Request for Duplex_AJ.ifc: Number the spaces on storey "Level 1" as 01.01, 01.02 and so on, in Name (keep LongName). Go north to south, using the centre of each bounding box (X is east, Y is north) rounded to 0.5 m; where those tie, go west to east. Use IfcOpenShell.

First a look at what the model holds.

```python
import ifcopenshell
import ifcopenshell.util.element
import ifcopenshell.util.placement

model = ifcopenshell.open("Duplex_AJ.ifc")
print(model.schema)
storey = next(s for s in model.by_type("IfcBuildingStorey") if s.Name == "Level 1")
spaces = [e for e in ifcopenshell.util.element.get_decomposition(storey) if e.is_a("IfcSpace")]
for e in sorted(spaces, key=lambda e: e.id()):
    origin = ifcopenshell.util.placement.get_local_placement(e.ObjectPlacement)[:3, 3]
    print(e.id(), e.Name, e.LongName, origin.round(2) + 0.0, sep=" | ")
```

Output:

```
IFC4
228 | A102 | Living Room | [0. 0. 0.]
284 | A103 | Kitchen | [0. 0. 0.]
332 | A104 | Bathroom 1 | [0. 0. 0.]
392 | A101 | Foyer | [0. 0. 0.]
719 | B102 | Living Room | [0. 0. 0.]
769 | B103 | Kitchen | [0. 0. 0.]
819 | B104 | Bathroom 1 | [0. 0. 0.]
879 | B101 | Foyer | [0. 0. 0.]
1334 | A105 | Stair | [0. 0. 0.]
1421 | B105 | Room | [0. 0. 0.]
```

```python
import ifcopenshell
import ifcopenshell.geom
import ifcopenshell.util.element
import ifcopenshell.util.shape

model = ifcopenshell.open("Duplex_AJ.ifc")
settings = ifcopenshell.geom.settings()
settings.set("use-world-coords", True)


def centre(element):
    shape = ifcopenshell.geom.create_shape(settings, element)
    return ifcopenshell.util.shape.get_bbox_centroid(shape.geometry)


storey = next(s for s in model.by_type("IfcBuildingStorey") if s.Name == "Level 1")
spaces = [e for e in ifcopenshell.util.element.get_decomposition(storey) if e.is_a("IfcSpace")]

# Insertion points can sit at a corner or the storey origin, so sort by the geometry (in metres).
centres = {e: centre(e) for e in spaces}
spaces.sort(key=lambda e: (-round(centres[e][1] / 0.5), centres[e][0]))

for i, e in enumerate(spaces, start=1):
    number = f"01.{i:02d}"
    e.Name = number
    print(e.id(), number)

model.write("Duplex_AJ_updated.ifc")
```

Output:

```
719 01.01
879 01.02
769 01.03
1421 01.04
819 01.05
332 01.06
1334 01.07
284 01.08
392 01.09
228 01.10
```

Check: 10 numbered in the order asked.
